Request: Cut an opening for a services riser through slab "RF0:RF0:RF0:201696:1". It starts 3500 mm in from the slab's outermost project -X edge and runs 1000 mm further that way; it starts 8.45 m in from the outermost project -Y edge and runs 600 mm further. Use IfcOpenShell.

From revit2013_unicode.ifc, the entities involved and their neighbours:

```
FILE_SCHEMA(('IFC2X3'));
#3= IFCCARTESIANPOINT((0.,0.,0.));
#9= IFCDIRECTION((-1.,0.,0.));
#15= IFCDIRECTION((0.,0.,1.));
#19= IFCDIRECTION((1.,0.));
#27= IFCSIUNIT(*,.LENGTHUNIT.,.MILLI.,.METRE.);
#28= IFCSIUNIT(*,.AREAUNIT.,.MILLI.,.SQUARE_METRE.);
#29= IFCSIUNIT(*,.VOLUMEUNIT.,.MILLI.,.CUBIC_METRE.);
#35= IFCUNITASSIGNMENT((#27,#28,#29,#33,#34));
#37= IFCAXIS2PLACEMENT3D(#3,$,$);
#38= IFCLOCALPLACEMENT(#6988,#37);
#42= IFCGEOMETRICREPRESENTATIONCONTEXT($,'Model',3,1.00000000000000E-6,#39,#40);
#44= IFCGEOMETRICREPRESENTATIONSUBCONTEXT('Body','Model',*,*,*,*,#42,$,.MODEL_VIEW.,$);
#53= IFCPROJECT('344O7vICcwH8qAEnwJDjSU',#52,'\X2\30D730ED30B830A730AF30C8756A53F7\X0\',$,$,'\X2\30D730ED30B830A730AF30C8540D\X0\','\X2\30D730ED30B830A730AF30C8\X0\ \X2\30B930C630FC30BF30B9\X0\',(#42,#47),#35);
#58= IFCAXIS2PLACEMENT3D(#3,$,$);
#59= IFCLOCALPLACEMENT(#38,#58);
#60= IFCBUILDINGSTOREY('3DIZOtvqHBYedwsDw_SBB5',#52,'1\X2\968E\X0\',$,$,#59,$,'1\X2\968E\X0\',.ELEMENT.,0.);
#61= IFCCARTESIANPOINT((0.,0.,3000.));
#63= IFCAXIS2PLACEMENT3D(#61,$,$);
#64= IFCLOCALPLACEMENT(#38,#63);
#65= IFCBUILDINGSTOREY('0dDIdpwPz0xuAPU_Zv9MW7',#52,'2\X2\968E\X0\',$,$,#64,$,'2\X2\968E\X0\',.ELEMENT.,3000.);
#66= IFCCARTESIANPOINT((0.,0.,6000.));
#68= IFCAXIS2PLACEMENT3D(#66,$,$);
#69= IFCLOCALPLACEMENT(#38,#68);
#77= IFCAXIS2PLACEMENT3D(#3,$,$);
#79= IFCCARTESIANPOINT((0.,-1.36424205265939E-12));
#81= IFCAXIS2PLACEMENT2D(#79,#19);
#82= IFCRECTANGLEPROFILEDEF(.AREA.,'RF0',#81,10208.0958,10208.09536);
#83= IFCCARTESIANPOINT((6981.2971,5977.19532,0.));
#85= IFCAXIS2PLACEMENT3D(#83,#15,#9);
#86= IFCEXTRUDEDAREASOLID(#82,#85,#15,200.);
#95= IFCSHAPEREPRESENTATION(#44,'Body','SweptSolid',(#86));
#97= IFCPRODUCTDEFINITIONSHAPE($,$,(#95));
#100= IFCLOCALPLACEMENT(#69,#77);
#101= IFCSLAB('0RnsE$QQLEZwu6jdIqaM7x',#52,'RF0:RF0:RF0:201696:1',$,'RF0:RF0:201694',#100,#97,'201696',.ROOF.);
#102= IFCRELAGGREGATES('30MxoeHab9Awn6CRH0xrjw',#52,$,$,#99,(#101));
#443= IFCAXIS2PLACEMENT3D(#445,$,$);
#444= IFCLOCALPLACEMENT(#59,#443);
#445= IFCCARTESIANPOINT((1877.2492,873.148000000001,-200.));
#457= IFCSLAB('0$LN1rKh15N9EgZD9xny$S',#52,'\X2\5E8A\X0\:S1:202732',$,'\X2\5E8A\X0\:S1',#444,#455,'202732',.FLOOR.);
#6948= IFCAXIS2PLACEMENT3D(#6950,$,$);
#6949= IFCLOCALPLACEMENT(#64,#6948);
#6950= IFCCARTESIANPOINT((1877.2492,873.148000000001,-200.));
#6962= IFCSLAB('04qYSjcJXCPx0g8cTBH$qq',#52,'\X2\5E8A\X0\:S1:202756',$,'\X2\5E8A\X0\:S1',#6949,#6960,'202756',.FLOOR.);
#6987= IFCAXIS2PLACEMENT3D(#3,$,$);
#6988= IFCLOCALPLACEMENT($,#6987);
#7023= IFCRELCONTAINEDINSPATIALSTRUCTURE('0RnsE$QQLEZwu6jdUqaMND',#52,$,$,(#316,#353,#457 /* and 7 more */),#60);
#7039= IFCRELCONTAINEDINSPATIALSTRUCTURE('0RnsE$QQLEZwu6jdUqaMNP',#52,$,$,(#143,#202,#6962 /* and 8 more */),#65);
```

```python
import numpy as np
import ifcopenshell
import ifcopenshell.api.feature
import ifcopenshell.api.geometry
import ifcopenshell.api.root
import ifcopenshell.geom
import ifcopenshell.util.placement
import ifcopenshell.util.representation
import ifcopenshell.util.shape
import ifcopenshell.util.unit

model = ifcopenshell.open("revit2013_unicode.ifc")
unit_scale = ifcopenshell.util.unit.calculate_unit_scale(model)
settings = ifcopenshell.geom.settings()


def volume(element):
    """Net volume in cubic metres, openings subtracted."""
    shape = ifcopenshell.geom.create_shape(settings, element)
    return ifcopenshell.util.shape.get_volume(shape.geometry)


slab = model.by_guid("0RnsE$QQLEZwu6jdIqaM7x")
before = volume(slab)

# Extent in the slab's own axes, in metres. The edges named are its -X and -Y sides.
slab_shape = ifcopenshell.geom.create_shape(settings, slab)
vertices = ifcopenshell.util.shape.get_vertices(slab_shape.geometry)
x_min, y_min, bottom = vertices.min(axis=0)
top = vertices[:, 2].max()

opening = ifcopenshell.api.root.create_entity(model, ifc_class="IfcOpeningElement", name="Services riser opening")
context = ifcopenshell.util.representation.get_context(model, "Model", "Body", "MODEL_VIEW")
width, depth = 1, 0.6
outline = [(0.0, 0.0), (width, 0.0), (width, depth), (0.0, depth), (0.0, 0.0)]
# Overshoot both faces by 50 mm so the cut is clean.
shape = ifcopenshell.api.geometry.add_slab_representation(
    model, context=context, depth=top - bottom + 0.1, polyline=outline
)
ifcopenshell.api.geometry.assign_representation(model, product=opening, representation=shape)

matrix = ifcopenshell.util.placement.get_local_placement(slab.ObjectPlacement)
matrix[:, 3] = matrix @ np.append(np.array([x_min + 3.5, y_min + 8.45, bottom - 0.05]) / unit_scale, 1.0)
ifcopenshell.api.geometry.edit_object_placement(model, product=opening, matrix=matrix, is_si=False)
ifcopenshell.api.feature.add_feature(model, feature=opening, element=slab)

after = volume(slab)

print(f"slab volume {before:.3f} -> {after:.3f} m3")

model.write("revit2013_unicode_rev.ifc")
```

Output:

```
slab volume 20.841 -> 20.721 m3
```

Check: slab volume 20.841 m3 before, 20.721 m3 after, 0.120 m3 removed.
